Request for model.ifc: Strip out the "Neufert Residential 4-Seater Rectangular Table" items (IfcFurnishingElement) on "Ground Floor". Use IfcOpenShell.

First a look at what the model holds.

```python
import ifcopenshell
import ifcopenshell.util.element

model = ifcopenshell.open("model.ifc")
print(model.schema)
storey = next(s for s in model.by_type("IfcBuildingStorey") if s.Name == "Ground Floor")
furniture = [e for e in ifcopenshell.util.element.get_decomposition(storey) if e.is_a("IfcFurnishingElement")]
seen = {}
for e in furniture:
    element_type = ifcopenshell.util.element.get_type(e)
    name = element_type.Name if element_type not in (None, e) else None
    seen[name] = seen.get(name, 0) + 1
for name, count in sorted(seen.items(), key=str):
    print(count, "x", name)
```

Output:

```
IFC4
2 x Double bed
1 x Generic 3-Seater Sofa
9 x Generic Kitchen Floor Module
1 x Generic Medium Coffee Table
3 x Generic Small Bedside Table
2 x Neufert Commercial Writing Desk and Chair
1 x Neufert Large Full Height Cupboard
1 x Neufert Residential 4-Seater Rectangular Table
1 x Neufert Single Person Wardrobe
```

```python
import ifcopenshell
import ifcopenshell.api.root
import ifcopenshell.util.element

model = ifcopenshell.open("model.ifc")

storey = next(s for s in model.by_type("IfcBuildingStorey") if s.Name == "Ground Floor")
furniture = [e for e in ifcopenshell.util.element.get_decomposition(storey) if e.is_a("IfcFurnishingElement")]
targets = [e for e in furniture if (t := ifcopenshell.util.element.get_type(e)) not in (None, e) and t.Name == "Neufert Residential 4-Seater Rectangular Table"]

for e in targets:
    ifcopenshell.api.root.remove_product(model, product=e)
print(len(targets), "removed")

model.write("model_v2.ifc")
```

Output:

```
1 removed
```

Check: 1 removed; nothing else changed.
